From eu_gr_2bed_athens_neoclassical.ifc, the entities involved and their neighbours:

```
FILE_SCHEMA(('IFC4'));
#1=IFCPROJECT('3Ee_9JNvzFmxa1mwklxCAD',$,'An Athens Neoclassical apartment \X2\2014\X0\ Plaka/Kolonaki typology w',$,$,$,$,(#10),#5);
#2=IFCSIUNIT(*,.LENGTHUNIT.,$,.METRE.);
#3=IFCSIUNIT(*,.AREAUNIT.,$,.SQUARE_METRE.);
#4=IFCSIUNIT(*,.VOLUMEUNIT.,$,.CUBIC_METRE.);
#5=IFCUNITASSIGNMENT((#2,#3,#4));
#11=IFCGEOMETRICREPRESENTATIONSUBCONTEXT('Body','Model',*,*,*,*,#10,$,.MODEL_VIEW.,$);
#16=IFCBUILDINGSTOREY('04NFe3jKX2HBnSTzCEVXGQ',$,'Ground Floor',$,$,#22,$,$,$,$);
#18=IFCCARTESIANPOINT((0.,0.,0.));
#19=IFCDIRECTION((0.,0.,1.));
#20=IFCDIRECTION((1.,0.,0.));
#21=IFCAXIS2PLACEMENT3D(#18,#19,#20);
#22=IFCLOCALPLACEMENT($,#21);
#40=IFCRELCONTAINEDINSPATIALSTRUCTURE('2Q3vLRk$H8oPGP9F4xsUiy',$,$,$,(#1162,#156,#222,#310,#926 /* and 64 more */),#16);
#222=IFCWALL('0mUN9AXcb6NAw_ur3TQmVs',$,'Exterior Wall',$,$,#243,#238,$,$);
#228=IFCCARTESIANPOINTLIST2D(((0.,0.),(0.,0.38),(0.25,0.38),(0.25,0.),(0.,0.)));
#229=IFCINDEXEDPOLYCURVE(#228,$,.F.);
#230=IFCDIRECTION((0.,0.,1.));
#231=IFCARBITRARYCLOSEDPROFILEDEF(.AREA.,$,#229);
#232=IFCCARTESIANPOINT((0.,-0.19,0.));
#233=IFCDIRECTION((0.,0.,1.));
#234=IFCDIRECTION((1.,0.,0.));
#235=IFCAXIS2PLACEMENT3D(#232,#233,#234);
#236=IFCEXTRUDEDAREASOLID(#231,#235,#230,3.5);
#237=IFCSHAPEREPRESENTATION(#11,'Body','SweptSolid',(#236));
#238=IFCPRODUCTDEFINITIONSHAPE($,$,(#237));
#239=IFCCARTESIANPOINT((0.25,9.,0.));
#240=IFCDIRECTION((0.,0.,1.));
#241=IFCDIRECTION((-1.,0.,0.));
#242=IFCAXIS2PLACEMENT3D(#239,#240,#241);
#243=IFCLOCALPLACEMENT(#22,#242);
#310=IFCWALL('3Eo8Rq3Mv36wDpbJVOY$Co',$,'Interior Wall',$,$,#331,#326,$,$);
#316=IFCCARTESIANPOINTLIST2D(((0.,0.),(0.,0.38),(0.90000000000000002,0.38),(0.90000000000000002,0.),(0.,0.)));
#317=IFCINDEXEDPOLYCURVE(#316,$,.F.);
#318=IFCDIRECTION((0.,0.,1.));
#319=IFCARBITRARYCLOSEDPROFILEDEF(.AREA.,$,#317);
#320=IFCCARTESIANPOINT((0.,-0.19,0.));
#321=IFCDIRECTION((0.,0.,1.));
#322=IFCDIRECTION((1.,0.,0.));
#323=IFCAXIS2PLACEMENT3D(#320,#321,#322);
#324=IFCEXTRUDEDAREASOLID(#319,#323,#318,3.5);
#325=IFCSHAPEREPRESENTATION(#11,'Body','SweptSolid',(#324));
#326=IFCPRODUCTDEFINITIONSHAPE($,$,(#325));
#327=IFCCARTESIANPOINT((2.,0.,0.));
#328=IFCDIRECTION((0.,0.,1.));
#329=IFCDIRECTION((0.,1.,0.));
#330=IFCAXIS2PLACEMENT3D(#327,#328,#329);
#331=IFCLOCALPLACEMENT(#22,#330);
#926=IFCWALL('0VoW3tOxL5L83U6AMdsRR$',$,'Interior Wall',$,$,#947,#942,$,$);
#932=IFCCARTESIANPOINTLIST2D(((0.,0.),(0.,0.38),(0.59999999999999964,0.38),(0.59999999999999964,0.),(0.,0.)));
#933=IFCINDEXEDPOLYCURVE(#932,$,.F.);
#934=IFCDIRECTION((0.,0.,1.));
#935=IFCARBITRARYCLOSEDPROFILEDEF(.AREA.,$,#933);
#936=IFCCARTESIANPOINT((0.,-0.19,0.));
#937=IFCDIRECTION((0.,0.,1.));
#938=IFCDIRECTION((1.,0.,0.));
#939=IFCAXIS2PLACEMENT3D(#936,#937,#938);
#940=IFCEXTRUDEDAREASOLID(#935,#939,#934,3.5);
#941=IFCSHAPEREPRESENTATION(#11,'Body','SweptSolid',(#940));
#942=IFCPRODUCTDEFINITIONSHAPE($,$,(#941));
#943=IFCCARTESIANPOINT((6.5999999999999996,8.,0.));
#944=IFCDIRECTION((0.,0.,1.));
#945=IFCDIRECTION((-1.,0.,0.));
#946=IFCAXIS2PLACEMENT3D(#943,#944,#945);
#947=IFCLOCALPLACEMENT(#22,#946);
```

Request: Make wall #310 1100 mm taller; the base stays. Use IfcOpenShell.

```python
import ifcopenshell
import ifcopenshell.geom
import ifcopenshell.util.representation
import ifcopenshell.util.shape

model = ifcopenshell.open("eu_gr_2bed_athens_neoclassical.ifc")
settings = ifcopenshell.geom.settings()


def volume(element):
    """Net volume in cubic metres, openings subtracted."""
    shape = ifcopenshell.geom.create_shape(settings, element)
    return ifcopenshell.util.shape.get_volume(shape.geometry)


wall = model.by_guid("3Eo8Rq3Mv36wDpbJVOY$Co")
before = volume(wall)

body = ifcopenshell.util.representation.get_representation(wall, "Model", "Body")
solid = body.Items[0]
old_height = solid.Depth
solid.Depth += 1.1
after = volume(wall)

print(f"height {old_height:g} -> {solid.Depth:g}, volume {before:.3f} -> {after:.3f} m3")

model.write("eu_gr_2bed_athens_neoclassical_edited.ifc")
```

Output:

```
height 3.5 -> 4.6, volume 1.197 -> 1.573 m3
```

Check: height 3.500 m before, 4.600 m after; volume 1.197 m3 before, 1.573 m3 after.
